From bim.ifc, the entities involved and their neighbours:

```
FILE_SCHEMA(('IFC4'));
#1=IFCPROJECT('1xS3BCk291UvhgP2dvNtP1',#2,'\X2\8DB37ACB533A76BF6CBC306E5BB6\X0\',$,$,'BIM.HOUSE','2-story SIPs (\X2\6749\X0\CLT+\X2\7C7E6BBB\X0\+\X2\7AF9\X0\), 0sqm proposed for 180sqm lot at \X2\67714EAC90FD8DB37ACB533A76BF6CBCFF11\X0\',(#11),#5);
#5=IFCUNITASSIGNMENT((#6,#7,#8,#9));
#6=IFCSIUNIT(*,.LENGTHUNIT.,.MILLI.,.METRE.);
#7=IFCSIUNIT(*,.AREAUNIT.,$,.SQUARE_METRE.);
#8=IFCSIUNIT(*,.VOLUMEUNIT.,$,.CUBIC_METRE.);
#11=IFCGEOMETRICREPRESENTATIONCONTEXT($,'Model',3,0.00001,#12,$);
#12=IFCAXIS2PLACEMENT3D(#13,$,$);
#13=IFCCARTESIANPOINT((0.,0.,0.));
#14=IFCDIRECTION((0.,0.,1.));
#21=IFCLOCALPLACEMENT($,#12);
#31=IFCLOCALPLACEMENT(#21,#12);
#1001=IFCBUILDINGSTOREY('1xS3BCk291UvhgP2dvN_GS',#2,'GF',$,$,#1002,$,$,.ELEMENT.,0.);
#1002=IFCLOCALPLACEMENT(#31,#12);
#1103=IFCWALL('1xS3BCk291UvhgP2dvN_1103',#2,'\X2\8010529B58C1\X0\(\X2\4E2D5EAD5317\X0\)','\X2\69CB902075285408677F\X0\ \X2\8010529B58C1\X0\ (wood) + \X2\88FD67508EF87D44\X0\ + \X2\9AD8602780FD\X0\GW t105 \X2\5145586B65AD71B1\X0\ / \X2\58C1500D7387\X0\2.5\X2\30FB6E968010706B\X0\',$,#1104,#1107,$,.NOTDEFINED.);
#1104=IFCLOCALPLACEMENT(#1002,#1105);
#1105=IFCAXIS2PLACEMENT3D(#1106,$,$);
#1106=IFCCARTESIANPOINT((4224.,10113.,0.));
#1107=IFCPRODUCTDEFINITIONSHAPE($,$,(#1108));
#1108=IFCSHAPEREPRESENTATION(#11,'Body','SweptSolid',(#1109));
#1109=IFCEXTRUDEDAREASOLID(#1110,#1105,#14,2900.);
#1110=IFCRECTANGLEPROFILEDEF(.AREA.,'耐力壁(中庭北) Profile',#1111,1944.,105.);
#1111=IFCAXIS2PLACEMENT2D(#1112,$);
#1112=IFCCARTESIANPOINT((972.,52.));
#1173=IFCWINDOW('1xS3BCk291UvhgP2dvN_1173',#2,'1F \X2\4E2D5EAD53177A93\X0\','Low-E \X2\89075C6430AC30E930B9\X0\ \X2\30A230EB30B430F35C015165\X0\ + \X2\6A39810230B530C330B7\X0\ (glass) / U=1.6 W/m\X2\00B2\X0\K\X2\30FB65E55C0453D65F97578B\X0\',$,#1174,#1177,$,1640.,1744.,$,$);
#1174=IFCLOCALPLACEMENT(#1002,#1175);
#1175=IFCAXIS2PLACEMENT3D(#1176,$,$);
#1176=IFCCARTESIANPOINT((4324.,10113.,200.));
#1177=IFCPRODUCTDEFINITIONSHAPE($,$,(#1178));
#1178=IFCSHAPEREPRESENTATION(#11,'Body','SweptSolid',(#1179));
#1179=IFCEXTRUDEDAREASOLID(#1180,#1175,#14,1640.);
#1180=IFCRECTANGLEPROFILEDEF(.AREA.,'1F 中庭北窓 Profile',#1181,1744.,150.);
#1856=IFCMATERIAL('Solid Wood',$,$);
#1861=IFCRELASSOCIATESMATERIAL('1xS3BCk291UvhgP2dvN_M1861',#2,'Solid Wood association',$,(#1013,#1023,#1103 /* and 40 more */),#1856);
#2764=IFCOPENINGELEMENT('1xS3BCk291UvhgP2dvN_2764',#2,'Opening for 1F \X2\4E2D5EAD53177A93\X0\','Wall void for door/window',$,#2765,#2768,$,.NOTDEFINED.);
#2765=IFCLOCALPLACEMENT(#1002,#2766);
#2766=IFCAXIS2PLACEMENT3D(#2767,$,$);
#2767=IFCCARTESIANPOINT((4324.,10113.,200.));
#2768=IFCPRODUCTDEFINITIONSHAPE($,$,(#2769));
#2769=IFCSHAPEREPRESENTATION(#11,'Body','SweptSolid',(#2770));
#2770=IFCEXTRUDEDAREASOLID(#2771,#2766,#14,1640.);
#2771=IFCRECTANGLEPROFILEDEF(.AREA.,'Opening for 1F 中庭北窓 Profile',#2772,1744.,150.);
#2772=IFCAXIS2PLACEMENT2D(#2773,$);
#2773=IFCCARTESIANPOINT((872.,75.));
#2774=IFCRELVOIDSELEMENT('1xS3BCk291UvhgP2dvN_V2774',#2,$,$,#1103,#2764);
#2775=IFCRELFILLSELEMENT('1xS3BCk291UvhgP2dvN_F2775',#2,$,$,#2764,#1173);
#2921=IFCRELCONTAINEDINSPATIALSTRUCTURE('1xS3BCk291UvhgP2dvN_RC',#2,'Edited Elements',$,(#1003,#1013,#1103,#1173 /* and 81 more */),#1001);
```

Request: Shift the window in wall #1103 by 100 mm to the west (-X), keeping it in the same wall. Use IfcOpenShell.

```python
import ifcopenshell
import ifcopenshell.api.geometry
import ifcopenshell.util.placement

model = ifcopenshell.open("bim.ifc")

window = model.by_id(1173)
opening = window.FillsVoids[0].RelatingOpeningElement
wall = opening.VoidsElements[0].RelatingBuildingElement

wall_matrix = ifcopenshell.util.placement.get_local_placement(wall.ObjectPlacement)
shift = wall_matrix[:3, 0] * -100.0
before = ifcopenshell.util.placement.get_local_placement(window.ObjectPlacement)[:3, 3].copy()

# The window is not placed relative to its opening, so move both.
for product in (opening, window):
    matrix = ifcopenshell.util.placement.get_local_placement(product.ObjectPlacement)
    matrix[:3, 3] += shift
    ifcopenshell.api.geometry.edit_object_placement(model, product=product, matrix=matrix, is_si=False)

after = ifcopenshell.util.placement.get_local_placement(window.ObjectPlacement)[:3, 3]
print("window moved by", (after - before).round(3) + 0.0)

model.write("bim_v2.ifc")
```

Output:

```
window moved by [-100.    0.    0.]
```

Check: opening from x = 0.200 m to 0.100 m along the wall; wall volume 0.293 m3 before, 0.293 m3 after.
